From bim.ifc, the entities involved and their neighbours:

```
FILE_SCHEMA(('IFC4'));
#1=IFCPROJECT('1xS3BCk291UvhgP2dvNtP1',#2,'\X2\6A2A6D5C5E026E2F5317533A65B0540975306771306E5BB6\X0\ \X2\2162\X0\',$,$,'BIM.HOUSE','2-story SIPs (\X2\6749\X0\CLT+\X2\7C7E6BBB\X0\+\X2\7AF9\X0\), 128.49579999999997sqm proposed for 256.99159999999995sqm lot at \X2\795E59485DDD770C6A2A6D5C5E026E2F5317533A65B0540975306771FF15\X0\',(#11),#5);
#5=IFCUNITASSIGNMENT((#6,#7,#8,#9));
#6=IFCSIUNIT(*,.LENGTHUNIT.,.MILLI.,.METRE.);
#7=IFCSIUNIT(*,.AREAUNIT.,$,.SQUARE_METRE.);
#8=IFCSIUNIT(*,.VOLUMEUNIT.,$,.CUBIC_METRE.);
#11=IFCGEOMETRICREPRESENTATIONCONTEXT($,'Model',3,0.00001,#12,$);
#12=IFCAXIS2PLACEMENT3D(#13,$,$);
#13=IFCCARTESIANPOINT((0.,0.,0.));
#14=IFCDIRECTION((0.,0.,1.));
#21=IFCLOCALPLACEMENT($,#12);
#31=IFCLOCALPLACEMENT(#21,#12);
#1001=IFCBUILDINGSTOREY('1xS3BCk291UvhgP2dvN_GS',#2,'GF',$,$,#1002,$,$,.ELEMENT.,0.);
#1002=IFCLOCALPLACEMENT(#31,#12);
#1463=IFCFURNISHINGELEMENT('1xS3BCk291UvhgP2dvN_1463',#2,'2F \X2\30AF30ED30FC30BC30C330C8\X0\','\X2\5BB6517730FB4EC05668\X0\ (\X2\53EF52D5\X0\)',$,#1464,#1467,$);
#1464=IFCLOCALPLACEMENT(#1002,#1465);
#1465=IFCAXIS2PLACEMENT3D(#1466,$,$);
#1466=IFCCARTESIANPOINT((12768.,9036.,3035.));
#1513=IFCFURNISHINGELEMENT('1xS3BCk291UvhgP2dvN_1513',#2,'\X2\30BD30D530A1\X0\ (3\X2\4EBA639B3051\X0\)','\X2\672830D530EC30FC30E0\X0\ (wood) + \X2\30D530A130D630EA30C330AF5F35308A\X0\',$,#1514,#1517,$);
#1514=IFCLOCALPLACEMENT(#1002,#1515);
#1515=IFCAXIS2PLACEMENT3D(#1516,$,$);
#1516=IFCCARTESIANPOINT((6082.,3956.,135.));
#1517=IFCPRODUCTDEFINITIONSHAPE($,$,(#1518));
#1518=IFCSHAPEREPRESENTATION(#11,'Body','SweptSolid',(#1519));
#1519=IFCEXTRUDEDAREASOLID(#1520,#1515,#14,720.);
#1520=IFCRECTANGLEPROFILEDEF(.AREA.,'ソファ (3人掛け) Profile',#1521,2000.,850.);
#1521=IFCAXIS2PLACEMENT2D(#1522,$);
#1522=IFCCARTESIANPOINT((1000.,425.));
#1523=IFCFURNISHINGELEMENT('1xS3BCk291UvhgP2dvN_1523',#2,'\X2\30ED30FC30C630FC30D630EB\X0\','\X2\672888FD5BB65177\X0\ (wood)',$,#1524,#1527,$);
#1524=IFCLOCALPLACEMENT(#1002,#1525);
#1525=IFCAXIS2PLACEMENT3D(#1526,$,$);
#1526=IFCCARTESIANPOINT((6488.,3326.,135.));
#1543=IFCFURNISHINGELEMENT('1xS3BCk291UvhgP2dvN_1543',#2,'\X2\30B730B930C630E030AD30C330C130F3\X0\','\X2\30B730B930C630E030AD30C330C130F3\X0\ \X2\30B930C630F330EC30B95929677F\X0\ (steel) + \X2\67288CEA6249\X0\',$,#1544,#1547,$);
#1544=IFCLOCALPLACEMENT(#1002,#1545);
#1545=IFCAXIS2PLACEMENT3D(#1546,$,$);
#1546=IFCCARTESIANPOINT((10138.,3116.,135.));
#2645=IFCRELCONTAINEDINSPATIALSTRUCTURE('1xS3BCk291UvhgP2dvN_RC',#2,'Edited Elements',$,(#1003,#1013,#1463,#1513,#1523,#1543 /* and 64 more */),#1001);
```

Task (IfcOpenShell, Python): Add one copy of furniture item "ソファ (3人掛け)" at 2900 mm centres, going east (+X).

```python
import numpy as np
import ifcopenshell
import ifcopenshell.api.geometry
import ifcopenshell.api.root
import ifcopenshell.util.element
import ifcopenshell.util.placement
import ifcopenshell.util.unit

model = ifcopenshell.open("bim.ifc")
unit_scale = ifcopenshell.util.unit.calculate_unit_scale(model)


def reuse_history(source, copy):
    """copy_class also copies each property set's owner history, people and application; keep the originals."""
    for rel in copy.IsDefinedBy:
        if rel.is_a("IfcRelDefinesByProperties") and (history := rel.RelatingPropertyDefinition.OwnerHistory):
            rel.RelatingPropertyDefinition.OwnerHistory = source.OwnerHistory
            ifcopenshell.util.element.remove_deep2(model, history)


source = model.by_guid("1xS3BCk291UvhgP2dvN_1513")
base = ifcopenshell.util.placement.get_local_placement(source.ObjectPlacement)
step = np.array([1.0, 0.0, 0.0]) * 2.9 / unit_scale

for i in range(1, 2):
    copy = ifcopenshell.api.root.copy_class(model, product=source)
    copy.Representation = ifcopenshell.util.element.copy_deep(
        model, source.Representation, exclude=["IfcGeometricRepresentationContext", "IfcRepresentationMap"]
    )
    reuse_history(source, copy)
    matrix = base.copy()
    matrix[:3, 3] += i * step
    print("added at", matrix[:3, 3].round(3) + 0.0)
    ifcopenshell.api.geometry.edit_object_placement(model, product=copy, matrix=matrix, is_si=False)

model.write("bim_updated.ifc")
```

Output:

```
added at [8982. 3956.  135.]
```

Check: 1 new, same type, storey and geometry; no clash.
